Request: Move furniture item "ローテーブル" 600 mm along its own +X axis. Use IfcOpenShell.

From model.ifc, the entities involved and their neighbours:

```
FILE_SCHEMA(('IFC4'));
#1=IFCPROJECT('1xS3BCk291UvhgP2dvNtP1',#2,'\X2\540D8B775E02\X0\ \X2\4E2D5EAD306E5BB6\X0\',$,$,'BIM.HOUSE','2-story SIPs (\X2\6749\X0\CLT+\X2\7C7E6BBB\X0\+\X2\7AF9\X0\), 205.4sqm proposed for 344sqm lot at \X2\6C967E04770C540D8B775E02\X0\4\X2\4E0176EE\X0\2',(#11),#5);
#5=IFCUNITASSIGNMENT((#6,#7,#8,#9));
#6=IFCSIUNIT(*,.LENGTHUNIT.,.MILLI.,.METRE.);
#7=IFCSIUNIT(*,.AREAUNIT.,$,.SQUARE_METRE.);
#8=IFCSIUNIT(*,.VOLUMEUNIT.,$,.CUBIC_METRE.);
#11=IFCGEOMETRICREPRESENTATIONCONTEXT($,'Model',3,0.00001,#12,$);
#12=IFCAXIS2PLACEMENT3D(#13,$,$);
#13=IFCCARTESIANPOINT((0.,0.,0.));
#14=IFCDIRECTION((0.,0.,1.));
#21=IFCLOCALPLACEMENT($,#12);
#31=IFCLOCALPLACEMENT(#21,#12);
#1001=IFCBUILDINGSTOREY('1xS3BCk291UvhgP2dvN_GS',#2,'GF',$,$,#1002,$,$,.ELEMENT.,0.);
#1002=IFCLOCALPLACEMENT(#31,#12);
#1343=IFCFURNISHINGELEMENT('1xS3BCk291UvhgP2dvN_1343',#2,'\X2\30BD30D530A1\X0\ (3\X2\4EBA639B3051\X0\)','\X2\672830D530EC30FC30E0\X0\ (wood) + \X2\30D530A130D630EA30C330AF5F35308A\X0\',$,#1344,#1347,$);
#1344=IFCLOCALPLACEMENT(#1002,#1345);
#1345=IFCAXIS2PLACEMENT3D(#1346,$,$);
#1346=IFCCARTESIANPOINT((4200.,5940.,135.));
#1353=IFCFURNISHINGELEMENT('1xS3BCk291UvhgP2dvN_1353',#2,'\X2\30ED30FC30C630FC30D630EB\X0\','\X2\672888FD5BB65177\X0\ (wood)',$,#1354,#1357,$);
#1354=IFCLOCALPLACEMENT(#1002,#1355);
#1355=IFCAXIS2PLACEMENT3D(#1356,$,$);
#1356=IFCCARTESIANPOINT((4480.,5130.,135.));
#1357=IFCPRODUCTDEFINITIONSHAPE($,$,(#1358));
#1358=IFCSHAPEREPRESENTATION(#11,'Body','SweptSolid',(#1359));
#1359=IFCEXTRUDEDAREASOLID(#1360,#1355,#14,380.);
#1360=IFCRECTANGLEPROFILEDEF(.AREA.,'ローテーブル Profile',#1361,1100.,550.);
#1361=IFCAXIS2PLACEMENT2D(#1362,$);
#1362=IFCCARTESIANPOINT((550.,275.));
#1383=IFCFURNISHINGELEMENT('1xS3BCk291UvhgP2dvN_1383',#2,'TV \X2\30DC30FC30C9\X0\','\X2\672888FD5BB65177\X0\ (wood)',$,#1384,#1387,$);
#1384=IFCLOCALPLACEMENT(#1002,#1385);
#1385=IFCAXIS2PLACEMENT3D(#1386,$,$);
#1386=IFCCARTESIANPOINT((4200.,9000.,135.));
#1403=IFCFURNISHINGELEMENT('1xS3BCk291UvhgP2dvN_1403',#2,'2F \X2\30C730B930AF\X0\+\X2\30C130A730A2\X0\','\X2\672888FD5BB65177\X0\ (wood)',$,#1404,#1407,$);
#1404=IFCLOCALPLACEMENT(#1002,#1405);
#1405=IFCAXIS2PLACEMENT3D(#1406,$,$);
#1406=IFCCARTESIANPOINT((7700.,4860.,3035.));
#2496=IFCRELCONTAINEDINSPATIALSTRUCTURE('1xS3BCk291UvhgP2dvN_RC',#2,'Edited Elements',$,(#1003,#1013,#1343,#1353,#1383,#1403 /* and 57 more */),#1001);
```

```python
import ifcopenshell
import ifcopenshell.api.geometry
import ifcopenshell.util.placement
import ifcopenshell.util.unit

model = ifcopenshell.open("model.ifc")
unit_scale = ifcopenshell.util.unit.calculate_unit_scale(model)

item = model.by_id(1353)
matrix = ifcopenshell.util.placement.get_local_placement(item.ObjectPlacement)
matrix[:3, 3] += matrix[:3, 0] * 0.6 / unit_scale
ifcopenshell.api.geometry.edit_object_placement(model, product=item, matrix=matrix, is_si=False)

print(ifcopenshell.util.placement.get_local_placement(item.ObjectPlacement).round(3) + 0.0)

model.write("model-out.ifc")
```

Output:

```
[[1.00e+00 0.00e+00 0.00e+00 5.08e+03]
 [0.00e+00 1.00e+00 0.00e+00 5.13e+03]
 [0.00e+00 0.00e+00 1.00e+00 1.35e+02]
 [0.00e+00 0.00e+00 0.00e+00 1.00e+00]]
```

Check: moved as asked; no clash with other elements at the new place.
